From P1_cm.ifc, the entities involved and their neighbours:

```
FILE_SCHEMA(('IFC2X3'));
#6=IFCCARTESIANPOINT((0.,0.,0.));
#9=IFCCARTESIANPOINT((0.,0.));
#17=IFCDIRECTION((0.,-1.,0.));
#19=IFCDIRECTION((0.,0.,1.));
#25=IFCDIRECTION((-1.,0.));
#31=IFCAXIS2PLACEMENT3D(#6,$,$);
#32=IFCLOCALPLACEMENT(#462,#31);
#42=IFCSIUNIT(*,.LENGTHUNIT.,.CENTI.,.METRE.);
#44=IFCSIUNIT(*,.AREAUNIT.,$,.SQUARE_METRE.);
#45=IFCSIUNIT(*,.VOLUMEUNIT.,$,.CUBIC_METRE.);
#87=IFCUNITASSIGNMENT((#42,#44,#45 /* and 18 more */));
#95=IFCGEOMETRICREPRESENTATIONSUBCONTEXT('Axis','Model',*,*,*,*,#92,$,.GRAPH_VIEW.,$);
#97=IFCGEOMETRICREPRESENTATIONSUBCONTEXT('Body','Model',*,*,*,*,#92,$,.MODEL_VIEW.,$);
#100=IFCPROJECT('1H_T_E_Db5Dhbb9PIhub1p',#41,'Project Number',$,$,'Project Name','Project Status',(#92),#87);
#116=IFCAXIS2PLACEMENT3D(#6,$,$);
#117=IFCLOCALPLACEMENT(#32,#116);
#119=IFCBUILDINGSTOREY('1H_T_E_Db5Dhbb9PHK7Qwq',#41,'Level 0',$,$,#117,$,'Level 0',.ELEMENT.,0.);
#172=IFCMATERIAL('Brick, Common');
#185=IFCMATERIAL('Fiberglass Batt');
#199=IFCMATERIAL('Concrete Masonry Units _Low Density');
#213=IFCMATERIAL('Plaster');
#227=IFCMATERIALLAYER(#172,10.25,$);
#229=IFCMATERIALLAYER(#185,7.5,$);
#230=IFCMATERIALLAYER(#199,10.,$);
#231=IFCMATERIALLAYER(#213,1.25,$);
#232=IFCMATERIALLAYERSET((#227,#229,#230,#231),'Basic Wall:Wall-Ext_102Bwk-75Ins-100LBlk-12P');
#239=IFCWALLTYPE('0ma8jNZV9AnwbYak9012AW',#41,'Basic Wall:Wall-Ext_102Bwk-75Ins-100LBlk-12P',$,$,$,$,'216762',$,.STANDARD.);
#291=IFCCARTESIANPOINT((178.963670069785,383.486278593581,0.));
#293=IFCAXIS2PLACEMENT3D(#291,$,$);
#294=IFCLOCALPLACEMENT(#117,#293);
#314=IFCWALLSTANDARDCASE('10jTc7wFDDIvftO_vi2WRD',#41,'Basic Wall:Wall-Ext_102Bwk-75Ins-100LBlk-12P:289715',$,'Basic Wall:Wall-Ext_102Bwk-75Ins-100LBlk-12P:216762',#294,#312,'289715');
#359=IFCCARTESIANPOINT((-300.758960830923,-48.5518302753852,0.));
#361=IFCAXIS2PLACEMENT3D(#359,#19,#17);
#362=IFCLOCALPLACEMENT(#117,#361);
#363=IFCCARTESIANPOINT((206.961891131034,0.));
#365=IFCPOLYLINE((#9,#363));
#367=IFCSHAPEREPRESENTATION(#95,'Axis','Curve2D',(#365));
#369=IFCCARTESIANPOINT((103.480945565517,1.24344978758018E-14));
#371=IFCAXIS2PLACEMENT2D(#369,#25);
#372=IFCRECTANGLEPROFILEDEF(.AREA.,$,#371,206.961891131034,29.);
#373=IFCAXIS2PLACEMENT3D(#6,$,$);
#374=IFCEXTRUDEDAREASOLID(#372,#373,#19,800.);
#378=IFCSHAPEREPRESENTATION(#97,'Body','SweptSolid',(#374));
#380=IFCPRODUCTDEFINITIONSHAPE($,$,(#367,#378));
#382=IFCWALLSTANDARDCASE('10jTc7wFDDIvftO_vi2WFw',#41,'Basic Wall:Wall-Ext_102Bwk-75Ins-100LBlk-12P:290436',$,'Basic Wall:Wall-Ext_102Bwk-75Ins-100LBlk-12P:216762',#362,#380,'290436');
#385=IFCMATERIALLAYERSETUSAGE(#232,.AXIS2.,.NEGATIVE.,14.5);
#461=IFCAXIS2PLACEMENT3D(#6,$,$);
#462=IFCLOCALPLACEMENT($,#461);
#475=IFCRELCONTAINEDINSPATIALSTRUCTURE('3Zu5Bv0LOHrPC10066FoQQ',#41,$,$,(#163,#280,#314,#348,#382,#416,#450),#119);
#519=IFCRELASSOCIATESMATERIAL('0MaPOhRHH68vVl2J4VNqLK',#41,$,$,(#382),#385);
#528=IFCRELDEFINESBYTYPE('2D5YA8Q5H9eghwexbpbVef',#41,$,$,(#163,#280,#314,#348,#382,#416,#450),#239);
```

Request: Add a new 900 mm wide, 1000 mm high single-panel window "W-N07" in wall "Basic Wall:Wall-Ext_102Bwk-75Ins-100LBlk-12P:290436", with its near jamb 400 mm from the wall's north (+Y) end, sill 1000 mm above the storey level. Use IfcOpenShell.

```python
import numpy as np
import ifcopenshell
import ifcopenshell.api.feature
import ifcopenshell.api.geometry
import ifcopenshell.api.root
import ifcopenshell.api.spatial
import ifcopenshell.api.type
import ifcopenshell.geom
import ifcopenshell.util.element
import ifcopenshell.util.placement
import ifcopenshell.util.representation
import ifcopenshell.util.shape
import ifcopenshell.util.unit

model = ifcopenshell.open("P1_cm.ifc")
unit_scale = ifcopenshell.util.unit.calculate_unit_scale(model)
settings = ifcopenshell.geom.settings()


def volume(element):
    """Net volume in cubic metres, openings subtracted."""
    shape = ifcopenshell.geom.create_shape(settings, element)
    return ifcopenshell.util.shape.get_volume(shape.geometry)


wall = model.by_id(382)
storey = ifcopenshell.util.element.get_container(wall, ifc_class="IfcBuildingStorey")
context = ifcopenshell.util.representation.get_context(model, "Model", "Body", "MODEL_VIEW")
before = volume(wall)

width, height, from_end, sill = 0.9, 1, 0.4, 1  # metres

# The wall runs along its own X axis, and the end named is its -X end.
wall_shape = ifcopenshell.geom.create_shape(settings, wall)
x, y, z = ifcopenshell.util.shape.get_vertices(wall_shape.geometry).T
start = x.min() + from_end
face, thickness = float(y.min()), float(y.max() - y.min())
wall_matrix = ifcopenshell.util.placement.get_local_placement(wall.ObjectPlacement)
level = ifcopenshell.util.placement.get_local_placement(storey.ObjectPlacement)[2, 3]


def in_wall(x, y):
    """Placement at x, y metres in the wall's axes, at sill height."""
    matrix = wall_matrix.copy()
    matrix[:, 3] = wall_matrix @ np.array([x / unit_scale, y / unit_scale, 0.0, 1.0])
    matrix[2, 3] = level + sill / unit_scale
    return matrix


# Opening: a box that overshoots both wall faces by 50 mm.
opening = ifcopenshell.api.root.create_entity(model, ifc_class="IfcOpeningElement")
box = ifcopenshell.api.geometry.add_wall_representation(
    model, context=context, length=width, height=height, thickness=thickness + 0.1
)
ifcopenshell.api.geometry.assign_representation(model, product=opening, representation=box)
ifcopenshell.api.geometry.edit_object_placement(model, product=opening, matrix=in_wall(start, face - 0.05), is_si=False)
ifcopenshell.api.feature.add_feature(model, feature=opening, element=wall)

window = ifcopenshell.api.root.create_entity(model, ifc_class="IfcWindow", name="W-N07")
window.OverallWidth, window.OverallHeight = width / unit_scale, height / unit_scale
body = ifcopenshell.api.geometry.add_window_representation(
    model,
    context=context,
    overall_width=window.OverallWidth,
    overall_height=window.OverallHeight,
    partition_type="SINGLE_PANEL",
)
ifcopenshell.api.geometry.assign_representation(model, product=window, representation=body)
ifcopenshell.api.spatial.assign_container(model, products=[window], relating_structure=storey)
fills = ifcopenshell.api.feature.add_filling(model, opening=opening, element=window)
fills.OwnerHistory = window.OwnerHistory  # required in IFC2X3

# IFC2X3 keeps the operation on the window style.
style = ifcopenshell.api.root.create_entity(model, ifc_class="IfcWindowStyle", name="W-N07")
style.OperationType, style.ConstructionType = "SINGLE_PANEL", "NOTDEFINED"
style.ParameterTakesPrecedence = style.Sizeable = False
ifcopenshell.api.type.assign_type(model, related_objects=[window], relating_type=style)

# Centre the window in the wall's thickness.
ifcopenshell.api.geometry.edit_object_placement(model, product=window, matrix=in_wall(start, face), is_si=False)
window_shape = ifcopenshell.geom.create_shape(settings, window)
depth = ifcopenshell.util.shape.get_vertices(window_shape.geometry)[:, 1]
offset = face + thickness / 2 - (depth.min() + depth.max()) / 2
ifcopenshell.api.geometry.edit_object_placement(model, product=window, matrix=in_wall(start, offset), is_si=False)

after = volume(wall)

print(f"wall volume {before:.3f} -> {after:.3f} m3")

model.write("P1_cm_v2.ifc")
```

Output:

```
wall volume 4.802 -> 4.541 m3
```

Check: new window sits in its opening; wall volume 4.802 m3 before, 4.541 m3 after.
